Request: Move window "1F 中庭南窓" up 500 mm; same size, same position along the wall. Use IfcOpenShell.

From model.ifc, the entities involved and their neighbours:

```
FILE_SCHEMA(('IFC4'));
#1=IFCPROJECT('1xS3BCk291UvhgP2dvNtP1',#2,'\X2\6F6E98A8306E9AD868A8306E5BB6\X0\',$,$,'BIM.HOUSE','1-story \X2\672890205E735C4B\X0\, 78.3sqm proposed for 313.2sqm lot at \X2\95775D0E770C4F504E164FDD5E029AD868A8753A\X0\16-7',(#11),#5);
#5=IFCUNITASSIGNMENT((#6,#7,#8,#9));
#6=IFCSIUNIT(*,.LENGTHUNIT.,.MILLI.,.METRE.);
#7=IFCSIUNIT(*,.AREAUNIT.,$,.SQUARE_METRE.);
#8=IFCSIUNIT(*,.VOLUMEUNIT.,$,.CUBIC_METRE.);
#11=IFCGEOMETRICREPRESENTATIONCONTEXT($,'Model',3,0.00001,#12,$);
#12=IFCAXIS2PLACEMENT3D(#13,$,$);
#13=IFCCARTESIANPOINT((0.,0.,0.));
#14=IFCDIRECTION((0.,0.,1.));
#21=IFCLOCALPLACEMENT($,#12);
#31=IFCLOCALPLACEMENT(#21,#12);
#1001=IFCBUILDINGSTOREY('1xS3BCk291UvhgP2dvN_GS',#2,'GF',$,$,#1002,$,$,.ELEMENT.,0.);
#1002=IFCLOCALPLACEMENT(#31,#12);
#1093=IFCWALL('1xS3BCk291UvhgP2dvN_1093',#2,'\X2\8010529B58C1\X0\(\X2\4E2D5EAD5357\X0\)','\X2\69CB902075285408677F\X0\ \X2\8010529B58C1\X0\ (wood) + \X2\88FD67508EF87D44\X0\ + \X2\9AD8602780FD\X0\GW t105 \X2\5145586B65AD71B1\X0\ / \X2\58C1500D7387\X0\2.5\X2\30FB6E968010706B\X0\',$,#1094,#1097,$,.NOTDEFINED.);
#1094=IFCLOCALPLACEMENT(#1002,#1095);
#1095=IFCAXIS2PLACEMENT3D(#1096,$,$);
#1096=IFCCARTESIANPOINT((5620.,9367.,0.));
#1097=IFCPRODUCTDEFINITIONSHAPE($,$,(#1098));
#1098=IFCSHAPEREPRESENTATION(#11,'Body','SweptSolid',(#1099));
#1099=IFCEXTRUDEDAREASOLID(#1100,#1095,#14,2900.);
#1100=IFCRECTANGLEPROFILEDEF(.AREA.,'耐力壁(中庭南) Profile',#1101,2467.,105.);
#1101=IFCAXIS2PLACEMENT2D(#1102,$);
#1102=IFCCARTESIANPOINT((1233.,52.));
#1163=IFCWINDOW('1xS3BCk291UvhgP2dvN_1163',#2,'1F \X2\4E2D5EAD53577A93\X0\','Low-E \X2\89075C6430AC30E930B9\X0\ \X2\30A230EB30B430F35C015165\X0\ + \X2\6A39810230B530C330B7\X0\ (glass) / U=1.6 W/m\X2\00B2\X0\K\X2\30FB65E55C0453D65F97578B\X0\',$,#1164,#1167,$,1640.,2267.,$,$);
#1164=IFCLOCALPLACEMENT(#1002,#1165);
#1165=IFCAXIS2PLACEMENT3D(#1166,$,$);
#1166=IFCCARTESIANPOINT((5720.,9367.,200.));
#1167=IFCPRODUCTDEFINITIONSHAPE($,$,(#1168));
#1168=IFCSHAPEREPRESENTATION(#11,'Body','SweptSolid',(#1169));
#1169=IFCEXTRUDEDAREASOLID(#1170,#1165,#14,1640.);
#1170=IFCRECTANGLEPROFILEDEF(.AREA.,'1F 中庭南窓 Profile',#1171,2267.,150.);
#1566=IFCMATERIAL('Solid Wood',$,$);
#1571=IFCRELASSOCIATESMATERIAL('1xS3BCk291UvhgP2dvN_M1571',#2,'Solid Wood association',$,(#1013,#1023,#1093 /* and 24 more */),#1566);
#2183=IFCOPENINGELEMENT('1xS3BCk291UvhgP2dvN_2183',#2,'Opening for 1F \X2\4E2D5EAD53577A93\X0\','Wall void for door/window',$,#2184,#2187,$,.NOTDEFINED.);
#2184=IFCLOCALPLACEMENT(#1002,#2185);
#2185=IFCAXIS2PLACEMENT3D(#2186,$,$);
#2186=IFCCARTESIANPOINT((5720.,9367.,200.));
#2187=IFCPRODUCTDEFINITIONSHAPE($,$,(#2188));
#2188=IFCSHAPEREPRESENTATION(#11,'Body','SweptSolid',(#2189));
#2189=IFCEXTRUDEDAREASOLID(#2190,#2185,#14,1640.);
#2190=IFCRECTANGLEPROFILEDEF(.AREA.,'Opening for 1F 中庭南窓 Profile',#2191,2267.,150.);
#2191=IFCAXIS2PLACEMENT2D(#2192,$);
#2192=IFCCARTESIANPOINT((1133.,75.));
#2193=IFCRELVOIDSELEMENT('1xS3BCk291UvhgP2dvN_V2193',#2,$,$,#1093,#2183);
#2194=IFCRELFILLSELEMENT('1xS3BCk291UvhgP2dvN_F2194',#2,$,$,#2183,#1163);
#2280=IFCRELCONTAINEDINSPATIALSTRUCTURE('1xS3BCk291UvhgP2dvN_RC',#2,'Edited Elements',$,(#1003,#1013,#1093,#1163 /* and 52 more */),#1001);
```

```python
import numpy as np
import ifcopenshell
import ifcopenshell.api.geometry
import ifcopenshell.util.placement
import ifcopenshell.util.unit

model = ifcopenshell.open("model.ifc")
unit_scale = ifcopenshell.util.unit.calculate_unit_scale(model)

window = model.by_guid("1xS3BCk291UvhgP2dvN_1163")
opening = window.FillsVoids[0].RelatingOpeningElement
dz = 0.5 / unit_scale

shift = np.array([0.0, 0.0, dz])
# The window is not placed relative to its opening, so move both.
for product in (opening, window):
    matrix = ifcopenshell.util.placement.get_local_placement(product.ObjectPlacement)
    matrix[:3, 3] += shift
    ifcopenshell.api.geometry.edit_object_placement(model, product=product, matrix=matrix, is_si=False)

print(f"moved by {dz * unit_scale:+.3f} m")

model.write("model-out.ifc")
```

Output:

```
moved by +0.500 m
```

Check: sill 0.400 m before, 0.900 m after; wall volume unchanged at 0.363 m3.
